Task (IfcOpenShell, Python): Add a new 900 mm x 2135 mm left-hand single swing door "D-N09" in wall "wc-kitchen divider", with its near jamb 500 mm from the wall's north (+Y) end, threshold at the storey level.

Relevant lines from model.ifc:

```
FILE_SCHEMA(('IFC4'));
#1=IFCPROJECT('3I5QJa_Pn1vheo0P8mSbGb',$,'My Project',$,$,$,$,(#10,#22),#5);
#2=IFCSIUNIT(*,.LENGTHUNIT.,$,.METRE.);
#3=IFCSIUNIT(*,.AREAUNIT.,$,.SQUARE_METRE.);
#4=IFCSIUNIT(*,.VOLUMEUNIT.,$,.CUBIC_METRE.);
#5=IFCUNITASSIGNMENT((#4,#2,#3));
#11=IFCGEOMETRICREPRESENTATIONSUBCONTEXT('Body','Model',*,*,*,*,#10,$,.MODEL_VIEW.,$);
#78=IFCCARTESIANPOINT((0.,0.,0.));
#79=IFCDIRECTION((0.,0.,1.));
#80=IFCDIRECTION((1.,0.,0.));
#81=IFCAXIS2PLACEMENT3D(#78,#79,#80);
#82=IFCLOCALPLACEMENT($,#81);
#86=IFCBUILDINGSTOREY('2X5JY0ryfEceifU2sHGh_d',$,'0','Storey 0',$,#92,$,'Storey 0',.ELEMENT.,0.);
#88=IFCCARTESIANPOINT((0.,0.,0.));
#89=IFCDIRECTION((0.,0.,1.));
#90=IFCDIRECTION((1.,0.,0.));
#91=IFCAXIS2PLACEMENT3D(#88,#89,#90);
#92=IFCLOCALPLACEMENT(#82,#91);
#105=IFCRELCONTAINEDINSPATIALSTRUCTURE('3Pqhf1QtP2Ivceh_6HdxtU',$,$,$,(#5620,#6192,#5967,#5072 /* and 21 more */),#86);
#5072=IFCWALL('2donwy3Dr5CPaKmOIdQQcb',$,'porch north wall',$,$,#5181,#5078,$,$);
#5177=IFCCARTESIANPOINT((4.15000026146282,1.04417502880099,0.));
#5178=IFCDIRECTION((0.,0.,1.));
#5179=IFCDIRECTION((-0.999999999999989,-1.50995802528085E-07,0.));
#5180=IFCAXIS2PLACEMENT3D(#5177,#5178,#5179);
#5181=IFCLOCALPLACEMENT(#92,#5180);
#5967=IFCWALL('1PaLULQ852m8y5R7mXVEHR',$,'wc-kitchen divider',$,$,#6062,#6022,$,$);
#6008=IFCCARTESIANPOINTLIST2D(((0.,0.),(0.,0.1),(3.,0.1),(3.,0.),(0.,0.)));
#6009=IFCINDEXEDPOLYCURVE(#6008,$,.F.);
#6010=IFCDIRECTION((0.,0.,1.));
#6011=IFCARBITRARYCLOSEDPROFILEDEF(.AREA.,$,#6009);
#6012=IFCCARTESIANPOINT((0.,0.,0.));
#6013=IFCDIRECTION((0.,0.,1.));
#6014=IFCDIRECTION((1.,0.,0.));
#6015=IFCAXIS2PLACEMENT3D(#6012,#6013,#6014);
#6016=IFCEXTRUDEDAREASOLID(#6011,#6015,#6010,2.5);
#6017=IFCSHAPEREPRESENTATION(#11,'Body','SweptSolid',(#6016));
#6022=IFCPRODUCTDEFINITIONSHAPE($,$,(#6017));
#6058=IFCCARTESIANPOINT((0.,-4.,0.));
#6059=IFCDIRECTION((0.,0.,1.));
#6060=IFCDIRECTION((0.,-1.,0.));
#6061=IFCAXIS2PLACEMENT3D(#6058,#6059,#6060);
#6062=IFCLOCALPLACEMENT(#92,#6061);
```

```python
import numpy as np
import ifcopenshell
import ifcopenshell.api.feature
import ifcopenshell.api.geometry
import ifcopenshell.api.root
import ifcopenshell.api.spatial
import ifcopenshell.geom
import ifcopenshell.util.element
import ifcopenshell.util.placement
import ifcopenshell.util.representation
import ifcopenshell.util.shape
import ifcopenshell.util.unit

model = ifcopenshell.open("model.ifc")
unit_scale = ifcopenshell.util.unit.calculate_unit_scale(model)
settings = ifcopenshell.geom.settings()


def volume(element):
    """Net volume in cubic metres, openings subtracted."""
    shape = ifcopenshell.geom.create_shape(settings, element)
    return ifcopenshell.util.shape.get_volume(shape.geometry)


wall = model.by_id(5967)
storey = ifcopenshell.util.element.get_container(wall, ifc_class="IfcBuildingStorey")
context = ifcopenshell.util.representation.get_context(model, "Model", "Body", "MODEL_VIEW")
before = volume(wall)

width, height, from_end, sill = 0.9, 2.135, 0.5, 0.0  # metres

# The wall runs along its own X axis, and the end named is its -X end.
wall_shape = ifcopenshell.geom.create_shape(settings, wall)
x, y, z = ifcopenshell.util.shape.get_vertices(wall_shape.geometry).T
start = x.min() + from_end
face, thickness = float(y.min()), float(y.max() - y.min())
wall_matrix = ifcopenshell.util.placement.get_local_placement(wall.ObjectPlacement)
level = ifcopenshell.util.placement.get_local_placement(storey.ObjectPlacement)[2, 3]


def in_wall(x, y):
    """Placement at x, y metres in the wall's axes, at sill height."""
    matrix = wall_matrix.copy()
    matrix[:, 3] = wall_matrix @ np.array([x / unit_scale, y / unit_scale, 0.0, 1.0])
    matrix[2, 3] = level + sill / unit_scale
    return matrix


# Opening: a box that overshoots both wall faces by 50 mm.
opening = ifcopenshell.api.root.create_entity(model, ifc_class="IfcOpeningElement", predefined_type="OPENING")
box = ifcopenshell.api.geometry.add_wall_representation(
    model, context=context, length=width, height=height, thickness=thickness + 0.1
)
ifcopenshell.api.geometry.assign_representation(model, product=opening, representation=box)
ifcopenshell.api.geometry.edit_object_placement(model, product=opening, matrix=in_wall(start, face - 0.05), is_si=False)
ifcopenshell.api.feature.add_feature(model, feature=opening, element=wall)

door = ifcopenshell.api.root.create_entity(model, ifc_class="IfcDoor", name="D-N09", predefined_type="DOOR")
door.OverallWidth, door.OverallHeight = width / unit_scale, height / unit_scale
door.OperationType = "SINGLE_SWING_LEFT"
body = ifcopenshell.api.geometry.add_door_representation(
    model,
    context=context,
    overall_width=door.OverallWidth,
    overall_height=door.OverallHeight,
    operation_type="SINGLE_SWING_LEFT",
    lining_properties={"LiningDepth": thickness / unit_scale, "ThresholdDepth": thickness / unit_scale},
)
ifcopenshell.api.geometry.assign_representation(model, product=door, representation=body)
ifcopenshell.api.spatial.assign_container(model, products=[door], relating_structure=storey)
ifcopenshell.api.feature.add_filling(model, opening=opening, element=door)

# The lining spans the wall, so the door starts at the wall face.
ifcopenshell.api.geometry.edit_object_placement(model, product=door, matrix=in_wall(start, face), is_si=False)

after = volume(wall)

print(f"wall volume {before:.3f} -> {after:.3f} m3")

model.write("model-out.ifc")
```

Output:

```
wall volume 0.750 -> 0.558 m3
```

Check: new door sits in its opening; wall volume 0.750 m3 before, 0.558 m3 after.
